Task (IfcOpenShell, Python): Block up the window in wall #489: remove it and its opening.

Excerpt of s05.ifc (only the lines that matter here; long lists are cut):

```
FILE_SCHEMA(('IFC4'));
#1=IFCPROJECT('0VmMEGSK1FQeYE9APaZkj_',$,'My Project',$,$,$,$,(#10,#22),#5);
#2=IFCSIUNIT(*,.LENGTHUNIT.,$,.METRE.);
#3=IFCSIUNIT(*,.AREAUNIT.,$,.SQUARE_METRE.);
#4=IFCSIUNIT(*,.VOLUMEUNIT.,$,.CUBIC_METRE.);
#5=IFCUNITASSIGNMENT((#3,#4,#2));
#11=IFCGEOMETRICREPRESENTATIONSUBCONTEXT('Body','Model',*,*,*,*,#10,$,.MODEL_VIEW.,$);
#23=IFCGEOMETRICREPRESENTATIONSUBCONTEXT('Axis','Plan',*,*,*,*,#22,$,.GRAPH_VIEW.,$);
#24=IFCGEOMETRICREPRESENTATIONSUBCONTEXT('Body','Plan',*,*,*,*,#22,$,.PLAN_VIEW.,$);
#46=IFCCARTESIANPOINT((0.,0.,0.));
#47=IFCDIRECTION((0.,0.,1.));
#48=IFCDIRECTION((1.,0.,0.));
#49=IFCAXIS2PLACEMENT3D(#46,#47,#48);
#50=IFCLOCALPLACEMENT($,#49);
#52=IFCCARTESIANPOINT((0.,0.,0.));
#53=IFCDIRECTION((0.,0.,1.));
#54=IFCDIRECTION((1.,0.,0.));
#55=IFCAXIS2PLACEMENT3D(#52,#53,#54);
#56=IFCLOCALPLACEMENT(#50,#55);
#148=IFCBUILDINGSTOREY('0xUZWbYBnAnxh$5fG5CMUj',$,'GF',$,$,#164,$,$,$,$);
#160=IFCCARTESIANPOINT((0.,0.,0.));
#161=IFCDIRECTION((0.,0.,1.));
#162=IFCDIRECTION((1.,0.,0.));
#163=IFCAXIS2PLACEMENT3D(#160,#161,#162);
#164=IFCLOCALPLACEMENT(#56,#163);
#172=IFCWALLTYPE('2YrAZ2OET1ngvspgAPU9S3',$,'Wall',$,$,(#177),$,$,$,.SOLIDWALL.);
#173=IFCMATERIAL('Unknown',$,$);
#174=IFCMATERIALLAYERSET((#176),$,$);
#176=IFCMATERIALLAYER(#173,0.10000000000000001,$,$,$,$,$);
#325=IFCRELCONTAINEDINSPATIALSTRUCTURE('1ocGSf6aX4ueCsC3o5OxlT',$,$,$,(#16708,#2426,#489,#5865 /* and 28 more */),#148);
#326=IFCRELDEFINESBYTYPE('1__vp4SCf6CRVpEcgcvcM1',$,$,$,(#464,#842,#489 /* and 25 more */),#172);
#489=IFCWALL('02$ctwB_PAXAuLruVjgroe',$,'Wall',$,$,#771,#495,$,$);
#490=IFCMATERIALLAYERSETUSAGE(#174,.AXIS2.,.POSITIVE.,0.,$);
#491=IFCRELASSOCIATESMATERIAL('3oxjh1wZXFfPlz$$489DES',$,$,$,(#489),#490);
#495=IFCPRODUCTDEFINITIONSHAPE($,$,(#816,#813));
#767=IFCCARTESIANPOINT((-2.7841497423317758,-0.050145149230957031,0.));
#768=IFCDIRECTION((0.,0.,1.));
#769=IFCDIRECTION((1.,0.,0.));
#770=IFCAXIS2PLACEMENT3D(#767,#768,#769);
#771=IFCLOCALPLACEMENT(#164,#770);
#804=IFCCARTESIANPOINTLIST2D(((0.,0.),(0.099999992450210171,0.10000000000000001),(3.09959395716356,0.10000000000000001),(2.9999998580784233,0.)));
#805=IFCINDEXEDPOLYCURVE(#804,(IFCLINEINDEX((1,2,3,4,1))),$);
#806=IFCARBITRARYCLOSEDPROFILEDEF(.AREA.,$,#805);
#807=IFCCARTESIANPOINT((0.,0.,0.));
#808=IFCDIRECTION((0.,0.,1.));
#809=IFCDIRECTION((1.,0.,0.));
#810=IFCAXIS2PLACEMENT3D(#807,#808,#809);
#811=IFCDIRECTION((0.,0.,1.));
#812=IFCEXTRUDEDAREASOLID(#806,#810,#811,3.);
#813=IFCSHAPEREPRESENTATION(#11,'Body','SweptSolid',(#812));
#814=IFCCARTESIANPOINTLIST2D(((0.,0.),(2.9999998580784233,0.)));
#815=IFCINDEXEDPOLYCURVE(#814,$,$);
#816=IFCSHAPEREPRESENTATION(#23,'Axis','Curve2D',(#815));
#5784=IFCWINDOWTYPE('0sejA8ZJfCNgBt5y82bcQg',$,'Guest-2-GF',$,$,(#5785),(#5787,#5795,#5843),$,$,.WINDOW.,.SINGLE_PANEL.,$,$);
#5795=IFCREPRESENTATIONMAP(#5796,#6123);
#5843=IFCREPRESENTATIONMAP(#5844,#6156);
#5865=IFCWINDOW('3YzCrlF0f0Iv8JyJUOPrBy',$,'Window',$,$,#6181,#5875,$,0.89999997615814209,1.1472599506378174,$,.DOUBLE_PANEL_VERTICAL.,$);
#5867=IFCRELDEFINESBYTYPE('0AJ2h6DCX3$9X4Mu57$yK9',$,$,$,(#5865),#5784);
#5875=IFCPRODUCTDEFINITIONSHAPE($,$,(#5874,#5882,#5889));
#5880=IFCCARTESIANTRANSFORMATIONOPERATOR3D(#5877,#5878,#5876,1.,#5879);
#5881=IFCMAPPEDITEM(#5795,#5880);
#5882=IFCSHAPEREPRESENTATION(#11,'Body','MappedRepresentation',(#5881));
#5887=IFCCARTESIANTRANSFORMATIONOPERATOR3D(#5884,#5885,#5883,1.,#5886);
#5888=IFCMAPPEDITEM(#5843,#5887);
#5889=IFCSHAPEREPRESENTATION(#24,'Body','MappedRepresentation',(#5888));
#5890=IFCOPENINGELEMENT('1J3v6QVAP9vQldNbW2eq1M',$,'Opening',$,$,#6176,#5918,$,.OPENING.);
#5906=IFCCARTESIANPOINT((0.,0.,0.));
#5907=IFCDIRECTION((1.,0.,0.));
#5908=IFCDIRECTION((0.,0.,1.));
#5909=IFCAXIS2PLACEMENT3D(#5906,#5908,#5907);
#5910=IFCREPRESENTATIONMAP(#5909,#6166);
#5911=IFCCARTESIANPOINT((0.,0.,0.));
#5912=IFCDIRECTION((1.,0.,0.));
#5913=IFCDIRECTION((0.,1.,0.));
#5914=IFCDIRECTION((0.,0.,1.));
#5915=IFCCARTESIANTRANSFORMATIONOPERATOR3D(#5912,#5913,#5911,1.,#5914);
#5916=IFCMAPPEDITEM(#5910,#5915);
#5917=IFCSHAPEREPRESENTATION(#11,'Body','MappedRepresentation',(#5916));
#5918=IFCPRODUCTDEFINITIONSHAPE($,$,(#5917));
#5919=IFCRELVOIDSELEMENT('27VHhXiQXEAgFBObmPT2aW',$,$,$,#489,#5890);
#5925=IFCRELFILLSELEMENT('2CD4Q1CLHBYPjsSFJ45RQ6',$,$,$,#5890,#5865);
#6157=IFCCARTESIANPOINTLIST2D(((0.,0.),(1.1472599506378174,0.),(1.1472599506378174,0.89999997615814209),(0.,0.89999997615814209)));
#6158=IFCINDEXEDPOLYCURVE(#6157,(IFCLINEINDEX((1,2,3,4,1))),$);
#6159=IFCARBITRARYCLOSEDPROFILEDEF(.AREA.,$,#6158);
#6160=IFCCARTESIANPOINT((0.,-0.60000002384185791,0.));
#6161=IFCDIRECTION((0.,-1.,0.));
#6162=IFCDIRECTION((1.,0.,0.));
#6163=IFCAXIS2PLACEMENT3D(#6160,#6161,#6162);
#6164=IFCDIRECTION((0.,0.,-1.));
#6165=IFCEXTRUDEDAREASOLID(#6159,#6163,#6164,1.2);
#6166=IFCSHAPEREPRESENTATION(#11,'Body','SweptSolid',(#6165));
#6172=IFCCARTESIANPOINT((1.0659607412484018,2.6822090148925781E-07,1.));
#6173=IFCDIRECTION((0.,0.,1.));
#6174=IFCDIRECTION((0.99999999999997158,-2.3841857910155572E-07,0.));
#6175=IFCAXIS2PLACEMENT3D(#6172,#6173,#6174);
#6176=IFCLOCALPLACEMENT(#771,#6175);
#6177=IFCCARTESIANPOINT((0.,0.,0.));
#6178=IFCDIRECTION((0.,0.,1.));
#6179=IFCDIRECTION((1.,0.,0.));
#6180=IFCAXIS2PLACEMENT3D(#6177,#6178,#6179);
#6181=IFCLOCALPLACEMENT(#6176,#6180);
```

```python
import ifcopenshell
import ifcopenshell.api.feature
import ifcopenshell.api.root
import ifcopenshell.geom
import ifcopenshell.util.shape

model = ifcopenshell.open("s05.ifc")
settings = ifcopenshell.geom.settings()


def volume(element):
    """Net volume in cubic metres, openings subtracted."""
    shape = ifcopenshell.geom.create_shape(settings, element)
    return ifcopenshell.util.shape.get_volume(shape.geometry)


window = model.by_guid("3YzCrlF0f0Iv8JyJUOPrBy")
opening = window.FillsVoids[0].RelatingOpeningElement
wall = opening.VoidsElements[0].RelatingBuildingElement
before = volume(wall)

ifcopenshell.api.root.remove_product(model, product=window)
ifcopenshell.api.feature.remove_feature(model, feature=opening)

after = volume(wall)

print(f"wall volume {before:.3f} -> {after:.3f} m3")

model.write("s05-out.ifc")
```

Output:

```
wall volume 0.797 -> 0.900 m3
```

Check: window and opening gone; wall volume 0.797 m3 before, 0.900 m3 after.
